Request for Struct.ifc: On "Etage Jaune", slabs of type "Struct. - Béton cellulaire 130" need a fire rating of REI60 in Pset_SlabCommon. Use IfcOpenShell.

First a look at what the model holds.

```python
import ifcopenshell
import ifcopenshell.util.element

model = ifcopenshell.open("Struct.ifc")
print(model.schema)
storey = next(s for s in model.by_type("IfcBuildingStorey") if s.Name == "Etage Jaune")
slabs = [e for e in ifcopenshell.util.element.get_decomposition(storey) if e.is_a("IfcSlab")]
seen = {}
for e in slabs:
    element_type = ifcopenshell.util.element.get_type(e)
    key = (element_type.Name if element_type != e and element_type else None, ifcopenshell.util.element.get_pset(e, "Pset_SlabCommon", "FireRating"))
    seen[key] = seen.get(key, 0) + 1
for (name, value), count in sorted(seen.items(), key=str):
    print(count, "x", name, "|", value)
```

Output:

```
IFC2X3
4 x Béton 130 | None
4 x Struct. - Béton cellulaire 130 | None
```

```python
import ifcopenshell
import ifcopenshell.api.pset
import ifcopenshell.util.element

model = ifcopenshell.open("Struct.ifc")

storey = next(s for s in model.by_type("IfcBuildingStorey") if s.Name == "Etage Jaune")
slabs = [e for e in ifcopenshell.util.element.get_decomposition(storey) if e.is_a("IfcSlab")]

count = 0
for e in slabs:
    element_type = ifcopenshell.util.element.get_type(e)
    if element_type in (None, e) or element_type.Name != "Struct. - Béton cellulaire 130":
        continue
    # add_pset returns the element's existing set when there is one.
    pset = ifcopenshell.api.pset.add_pset(model, product=e, name="Pset_SlabCommon")
    ifcopenshell.api.pset.edit_pset(model, pset=pset, properties={"FireRating": "REI60"})
    count += 1

print(count, "slabs updated")

model.write("Struct-out.ifc")
```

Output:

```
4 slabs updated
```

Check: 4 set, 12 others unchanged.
